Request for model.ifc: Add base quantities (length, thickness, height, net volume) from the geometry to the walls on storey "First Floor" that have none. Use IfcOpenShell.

First a look at what the model holds.

```python
import ifcopenshell
import ifcopenshell.util.element
import ifcopenshell.util.unit

model = ifcopenshell.open("model.ifc")
print(model.schema)
for unit_type in ("LENGTHUNIT", "AREAUNIT", "VOLUMEUNIT"):
    print(unit_type, ifcopenshell.util.unit.calculate_unit_scale(model, unit_type))
storey = next(s for s in model.by_type("IfcBuildingStorey") if s.Name == "First Floor")
walls = [e for e in ifcopenshell.util.element.get_decomposition(storey) if e.is_a("IfcWall")]
for e in sorted(walls, key=lambda e: e.id()):
    print(e.id(), e.is_a(), e.Name, list(ifcopenshell.util.element.get_psets(e, qtos_only=True)), sep=" | ")
```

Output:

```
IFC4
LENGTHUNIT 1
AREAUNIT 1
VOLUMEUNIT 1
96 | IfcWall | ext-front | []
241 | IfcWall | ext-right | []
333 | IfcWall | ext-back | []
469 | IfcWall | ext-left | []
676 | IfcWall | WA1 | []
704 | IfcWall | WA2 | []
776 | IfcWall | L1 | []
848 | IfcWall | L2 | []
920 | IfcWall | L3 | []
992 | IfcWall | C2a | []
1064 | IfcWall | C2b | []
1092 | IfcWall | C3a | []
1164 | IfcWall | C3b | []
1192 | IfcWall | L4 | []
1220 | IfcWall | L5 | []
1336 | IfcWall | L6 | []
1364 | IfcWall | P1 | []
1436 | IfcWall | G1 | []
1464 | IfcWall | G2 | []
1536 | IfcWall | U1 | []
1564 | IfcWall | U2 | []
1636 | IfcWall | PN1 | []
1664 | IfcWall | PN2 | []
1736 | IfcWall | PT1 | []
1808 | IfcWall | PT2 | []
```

```python
import ifcopenshell
import ifcopenshell.api.pset
import ifcopenshell.geom
import ifcopenshell.util.element
import ifcopenshell.util.shape
import ifcopenshell.util.unit

model = ifcopenshell.open("model.ifc")
unit_scale = ifcopenshell.util.unit.calculate_unit_scale(model)
volume_scale = ifcopenshell.util.unit.calculate_unit_scale(model, "VOLUMEUNIT")
settings = ifcopenshell.geom.settings()

storey = next(s for s in model.by_type("IfcBuildingStorey") if s.Name == "First Floor")
walls = [e for e in ifcopenshell.util.element.get_decomposition(storey) if e.is_a("IfcWall")]

for e in sorted(walls, key=lambda e: e.id()):
    if ifcopenshell.util.element.get_psets(e, qtos_only=True, should_inherit=False):
        continue
    # Geometry comes back in metres, in the element's own axes.
    shape = ifcopenshell.geom.create_shape(settings, e)
    values = {
        "Length": ifcopenshell.util.shape.get_x(shape.geometry) / unit_scale,
        "Width": ifcopenshell.util.shape.get_y(shape.geometry) / unit_scale,
        "Height": ifcopenshell.util.shape.get_z(shape.geometry) / unit_scale,
        "NetVolume": ifcopenshell.util.shape.get_volume(shape.geometry) / volume_scale,
    }
    qto = ifcopenshell.api.pset.add_qto(model, product=e, name="Qto_WallBaseQuantities")
    ifcopenshell.api.pset.edit_qto(model, qto=qto, properties=values)
    print(e.id(), {k: round(v, 3) for k, v in values.items()})

model.write("model-out.ifc")
```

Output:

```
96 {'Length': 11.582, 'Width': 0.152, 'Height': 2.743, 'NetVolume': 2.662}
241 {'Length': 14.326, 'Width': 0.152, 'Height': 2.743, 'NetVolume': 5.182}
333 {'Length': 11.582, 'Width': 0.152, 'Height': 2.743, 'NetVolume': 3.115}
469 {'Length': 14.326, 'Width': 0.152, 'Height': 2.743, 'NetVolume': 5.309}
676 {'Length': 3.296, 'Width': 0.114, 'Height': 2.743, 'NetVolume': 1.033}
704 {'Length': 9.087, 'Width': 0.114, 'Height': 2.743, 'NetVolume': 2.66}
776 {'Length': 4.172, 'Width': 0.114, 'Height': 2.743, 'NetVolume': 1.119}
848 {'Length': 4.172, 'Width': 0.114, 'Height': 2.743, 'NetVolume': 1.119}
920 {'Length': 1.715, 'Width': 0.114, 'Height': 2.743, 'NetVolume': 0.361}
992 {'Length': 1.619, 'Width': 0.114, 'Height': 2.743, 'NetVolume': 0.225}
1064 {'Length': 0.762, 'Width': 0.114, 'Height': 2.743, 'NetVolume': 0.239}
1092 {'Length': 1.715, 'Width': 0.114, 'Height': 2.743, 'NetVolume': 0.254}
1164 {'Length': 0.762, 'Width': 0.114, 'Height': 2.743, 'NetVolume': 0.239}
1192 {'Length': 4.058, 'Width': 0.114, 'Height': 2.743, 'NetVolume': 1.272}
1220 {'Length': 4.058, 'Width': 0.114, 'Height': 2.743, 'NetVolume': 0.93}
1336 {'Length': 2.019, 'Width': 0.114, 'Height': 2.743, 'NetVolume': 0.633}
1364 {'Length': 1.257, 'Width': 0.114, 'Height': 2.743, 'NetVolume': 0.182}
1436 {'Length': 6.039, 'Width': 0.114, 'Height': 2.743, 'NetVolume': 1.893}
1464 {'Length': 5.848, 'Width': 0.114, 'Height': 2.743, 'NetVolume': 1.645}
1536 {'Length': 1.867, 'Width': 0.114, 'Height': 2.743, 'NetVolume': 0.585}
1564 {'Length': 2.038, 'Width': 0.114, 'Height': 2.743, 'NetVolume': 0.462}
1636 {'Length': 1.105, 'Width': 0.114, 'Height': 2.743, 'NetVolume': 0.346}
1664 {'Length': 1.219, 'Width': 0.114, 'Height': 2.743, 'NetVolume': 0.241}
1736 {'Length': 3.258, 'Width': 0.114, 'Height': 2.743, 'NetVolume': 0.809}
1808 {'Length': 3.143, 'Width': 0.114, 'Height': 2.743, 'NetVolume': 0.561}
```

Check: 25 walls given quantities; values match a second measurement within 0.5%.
